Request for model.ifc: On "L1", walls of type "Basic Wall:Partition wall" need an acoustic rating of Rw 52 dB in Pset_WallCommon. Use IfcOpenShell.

First a look at what the model holds.

```python
import ifcopenshell
import ifcopenshell.util.element

model = ifcopenshell.open("model.ifc")
print(model.schema)
storey = next(s for s in model.by_type("IfcBuildingStorey") if s.Name == "L1")
walls = [e for e in ifcopenshell.util.element.get_decomposition(storey) if e.is_a("IfcWall")]
seen = {}
for e in walls:
    element_type = ifcopenshell.util.element.get_type(e)
    key = (element_type.Name if element_type != e and element_type else None, ifcopenshell.util.element.get_pset(e, "Pset_WallCommon", "AcousticRating"))
    seen[key] = seen.get(key, 0) + 1
for (name, value), count in sorted(seen.items(), key=str):
    print(count, "x", name, "|", value)
```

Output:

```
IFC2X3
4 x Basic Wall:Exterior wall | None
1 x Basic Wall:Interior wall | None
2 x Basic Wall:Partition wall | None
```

```python
import ifcopenshell
import ifcopenshell.api.pset
import ifcopenshell.util.element

model = ifcopenshell.open("model.ifc")

storey = next(s for s in model.by_type("IfcBuildingStorey") if s.Name == "L1")
walls = [e for e in ifcopenshell.util.element.get_decomposition(storey) if e.is_a("IfcWall")]

count = 0
for e in walls:
    element_type = ifcopenshell.util.element.get_type(e)
    if element_type in (None, e) or element_type.Name != "Basic Wall:Partition wall":
        continue
    # add_pset returns the element's existing set when there is one.
    pset = ifcopenshell.api.pset.add_pset(model, product=e, name="Pset_WallCommon")
    ifcopenshell.api.pset.edit_pset(model, pset=pset, properties={"AcousticRating": "Rw 52 dB"})
    count += 1

print(count, "walls updated")

model.write("model_edited.ifc")
```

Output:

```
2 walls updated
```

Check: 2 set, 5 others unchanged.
